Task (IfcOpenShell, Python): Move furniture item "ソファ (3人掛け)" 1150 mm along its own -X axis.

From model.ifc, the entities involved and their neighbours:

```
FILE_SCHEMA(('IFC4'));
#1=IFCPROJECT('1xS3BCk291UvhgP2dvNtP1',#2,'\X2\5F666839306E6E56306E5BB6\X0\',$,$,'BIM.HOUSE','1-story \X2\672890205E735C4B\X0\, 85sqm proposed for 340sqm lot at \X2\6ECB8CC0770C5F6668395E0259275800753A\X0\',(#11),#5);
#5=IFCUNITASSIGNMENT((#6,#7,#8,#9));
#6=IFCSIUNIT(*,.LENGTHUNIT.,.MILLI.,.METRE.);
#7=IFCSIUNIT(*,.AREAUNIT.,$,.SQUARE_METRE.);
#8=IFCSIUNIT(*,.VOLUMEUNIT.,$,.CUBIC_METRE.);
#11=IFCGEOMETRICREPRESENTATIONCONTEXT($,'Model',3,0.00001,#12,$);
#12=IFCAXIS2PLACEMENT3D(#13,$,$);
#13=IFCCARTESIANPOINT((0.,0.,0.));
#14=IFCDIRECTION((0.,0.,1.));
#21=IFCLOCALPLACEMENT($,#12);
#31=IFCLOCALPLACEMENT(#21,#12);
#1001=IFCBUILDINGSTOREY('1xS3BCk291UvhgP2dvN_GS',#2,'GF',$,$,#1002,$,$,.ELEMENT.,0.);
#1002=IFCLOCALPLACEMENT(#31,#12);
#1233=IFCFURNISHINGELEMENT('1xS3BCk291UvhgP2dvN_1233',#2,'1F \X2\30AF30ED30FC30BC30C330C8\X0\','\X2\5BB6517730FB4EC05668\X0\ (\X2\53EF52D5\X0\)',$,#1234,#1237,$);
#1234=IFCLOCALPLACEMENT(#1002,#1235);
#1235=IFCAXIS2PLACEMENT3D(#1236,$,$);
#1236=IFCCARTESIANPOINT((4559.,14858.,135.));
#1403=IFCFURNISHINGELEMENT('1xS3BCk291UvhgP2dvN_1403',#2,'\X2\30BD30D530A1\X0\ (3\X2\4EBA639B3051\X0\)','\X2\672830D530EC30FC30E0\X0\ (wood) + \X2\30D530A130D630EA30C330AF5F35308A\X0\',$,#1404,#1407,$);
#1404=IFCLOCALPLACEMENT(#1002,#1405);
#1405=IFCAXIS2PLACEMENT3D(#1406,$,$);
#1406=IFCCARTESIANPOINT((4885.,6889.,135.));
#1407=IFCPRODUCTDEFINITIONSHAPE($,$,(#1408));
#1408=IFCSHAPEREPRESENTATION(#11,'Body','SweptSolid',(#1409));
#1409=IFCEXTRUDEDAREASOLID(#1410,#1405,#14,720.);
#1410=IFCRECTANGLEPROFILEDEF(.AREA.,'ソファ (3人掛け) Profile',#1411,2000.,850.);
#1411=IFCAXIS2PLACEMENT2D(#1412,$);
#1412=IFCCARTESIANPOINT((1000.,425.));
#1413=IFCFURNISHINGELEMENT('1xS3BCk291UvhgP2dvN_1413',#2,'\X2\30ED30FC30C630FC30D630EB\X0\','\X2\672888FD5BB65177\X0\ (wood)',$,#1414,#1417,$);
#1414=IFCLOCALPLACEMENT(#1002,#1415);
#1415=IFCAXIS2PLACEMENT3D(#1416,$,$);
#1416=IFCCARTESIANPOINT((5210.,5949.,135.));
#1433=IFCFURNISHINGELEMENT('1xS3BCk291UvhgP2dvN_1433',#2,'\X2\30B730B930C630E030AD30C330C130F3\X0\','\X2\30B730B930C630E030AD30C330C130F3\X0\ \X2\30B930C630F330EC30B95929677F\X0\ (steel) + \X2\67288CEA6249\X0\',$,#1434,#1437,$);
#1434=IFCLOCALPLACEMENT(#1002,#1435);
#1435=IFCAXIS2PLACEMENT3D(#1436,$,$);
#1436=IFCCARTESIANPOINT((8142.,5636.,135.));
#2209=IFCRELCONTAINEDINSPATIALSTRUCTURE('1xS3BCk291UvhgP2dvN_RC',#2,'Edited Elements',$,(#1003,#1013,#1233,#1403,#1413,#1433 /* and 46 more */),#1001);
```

```python
import ifcopenshell
import ifcopenshell.api.geometry
import ifcopenshell.util.placement

model = ifcopenshell.open("model.ifc")

item = model.by_guid("1xS3BCk291UvhgP2dvN_1403")
matrix = ifcopenshell.util.placement.get_local_placement(item.ObjectPlacement)
matrix[:3, 3] -= matrix[:3, 0] * 1150.0
ifcopenshell.api.geometry.edit_object_placement(model, product=item, matrix=matrix, is_si=False)

print(ifcopenshell.util.placement.get_local_placement(item.ObjectPlacement).round(3) + 0.0)

model.write("model-out.ifc")
```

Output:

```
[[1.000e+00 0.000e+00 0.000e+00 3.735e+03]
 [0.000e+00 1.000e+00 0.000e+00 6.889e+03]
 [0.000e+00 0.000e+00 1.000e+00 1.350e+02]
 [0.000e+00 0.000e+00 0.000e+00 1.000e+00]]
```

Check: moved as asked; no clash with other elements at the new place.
